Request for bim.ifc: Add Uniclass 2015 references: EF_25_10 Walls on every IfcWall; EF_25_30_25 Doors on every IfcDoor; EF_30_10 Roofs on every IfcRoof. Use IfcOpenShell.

First a look at what the model holds.

```python
import ifcopenshell

model = ifcopenshell.open("bim.ifc")
print(model.schema)
print("classifications:", [c.Name for c in model.by_type("IfcClassification")])
for ifc_class in ("IfcDoor", "IfcRoof", "IfcStair", "IfcWall", "IfcWindow"):
    print(ifc_class, len(model.by_type(ifc_class)))
```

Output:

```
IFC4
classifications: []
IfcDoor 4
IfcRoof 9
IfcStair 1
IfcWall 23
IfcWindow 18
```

```python
import ifcopenshell
import ifcopenshell.api.classification

model = ifcopenshell.open("bim.ifc")

system = ifcopenshell.api.classification.add_classification(model, classification="Uniclass 2015")

codes = {
    "IfcWall": ("EF_25_10", "Walls"),
    "IfcDoor": ("EF_25_30_25", "Doors"),
    "IfcRoof": ("EF_30_10", "Roofs"),
}
for ifc_class, (code, name) in codes.items():
    products = model.by_type(ifc_class)
    ifcopenshell.api.classification.add_reference(
        model, products=products, classification=system, identification=code, name=name
    )
    print(code, len(products))

model.write("bim_v2.ifc")
```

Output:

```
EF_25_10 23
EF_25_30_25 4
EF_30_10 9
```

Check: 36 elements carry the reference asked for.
